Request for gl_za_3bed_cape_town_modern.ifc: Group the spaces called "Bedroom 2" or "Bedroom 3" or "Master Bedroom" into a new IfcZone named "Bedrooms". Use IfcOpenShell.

First a look at what the model holds.

```python
import ifcopenshell

model = ifcopenshell.open("gl_za_3bed_cape_town_modern.ifc")
print(model.schema)
seen = {}
for space in model.by_type("IfcSpace"):
    seen[space.LongName] = seen.get(space.LongName, 0) + 1
for name, count in sorted(seen.items(), key=str):
    print(count, "x", name)
print("zones:", [z.Name for z in model.by_type("IfcZone")][:20])
```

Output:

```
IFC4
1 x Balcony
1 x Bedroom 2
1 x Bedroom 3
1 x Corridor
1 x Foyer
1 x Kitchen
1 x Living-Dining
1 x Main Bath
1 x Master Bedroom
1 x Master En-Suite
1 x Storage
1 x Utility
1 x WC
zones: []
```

```python
import ifcopenshell
import ifcopenshell.api.group
import ifcopenshell.api.root

model = ifcopenshell.open("gl_za_3bed_cape_town_modern.ifc")

names = {"Bedroom 2", "Bedroom 3", "Master Bedroom"}
spaces = [s for s in model.by_type("IfcSpace") if s.LongName in names]

zone = ifcopenshell.api.root.create_entity(model, ifc_class="IfcZone", name="Bedrooms")
ifcopenshell.api.group.assign_group(model, products=spaces, group=zone)
print(len(spaces), "spaces in", zone.Name)

model.write("gl_za_3bed_cape_town_modern_edited.ifc")
```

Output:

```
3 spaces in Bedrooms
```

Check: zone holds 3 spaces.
